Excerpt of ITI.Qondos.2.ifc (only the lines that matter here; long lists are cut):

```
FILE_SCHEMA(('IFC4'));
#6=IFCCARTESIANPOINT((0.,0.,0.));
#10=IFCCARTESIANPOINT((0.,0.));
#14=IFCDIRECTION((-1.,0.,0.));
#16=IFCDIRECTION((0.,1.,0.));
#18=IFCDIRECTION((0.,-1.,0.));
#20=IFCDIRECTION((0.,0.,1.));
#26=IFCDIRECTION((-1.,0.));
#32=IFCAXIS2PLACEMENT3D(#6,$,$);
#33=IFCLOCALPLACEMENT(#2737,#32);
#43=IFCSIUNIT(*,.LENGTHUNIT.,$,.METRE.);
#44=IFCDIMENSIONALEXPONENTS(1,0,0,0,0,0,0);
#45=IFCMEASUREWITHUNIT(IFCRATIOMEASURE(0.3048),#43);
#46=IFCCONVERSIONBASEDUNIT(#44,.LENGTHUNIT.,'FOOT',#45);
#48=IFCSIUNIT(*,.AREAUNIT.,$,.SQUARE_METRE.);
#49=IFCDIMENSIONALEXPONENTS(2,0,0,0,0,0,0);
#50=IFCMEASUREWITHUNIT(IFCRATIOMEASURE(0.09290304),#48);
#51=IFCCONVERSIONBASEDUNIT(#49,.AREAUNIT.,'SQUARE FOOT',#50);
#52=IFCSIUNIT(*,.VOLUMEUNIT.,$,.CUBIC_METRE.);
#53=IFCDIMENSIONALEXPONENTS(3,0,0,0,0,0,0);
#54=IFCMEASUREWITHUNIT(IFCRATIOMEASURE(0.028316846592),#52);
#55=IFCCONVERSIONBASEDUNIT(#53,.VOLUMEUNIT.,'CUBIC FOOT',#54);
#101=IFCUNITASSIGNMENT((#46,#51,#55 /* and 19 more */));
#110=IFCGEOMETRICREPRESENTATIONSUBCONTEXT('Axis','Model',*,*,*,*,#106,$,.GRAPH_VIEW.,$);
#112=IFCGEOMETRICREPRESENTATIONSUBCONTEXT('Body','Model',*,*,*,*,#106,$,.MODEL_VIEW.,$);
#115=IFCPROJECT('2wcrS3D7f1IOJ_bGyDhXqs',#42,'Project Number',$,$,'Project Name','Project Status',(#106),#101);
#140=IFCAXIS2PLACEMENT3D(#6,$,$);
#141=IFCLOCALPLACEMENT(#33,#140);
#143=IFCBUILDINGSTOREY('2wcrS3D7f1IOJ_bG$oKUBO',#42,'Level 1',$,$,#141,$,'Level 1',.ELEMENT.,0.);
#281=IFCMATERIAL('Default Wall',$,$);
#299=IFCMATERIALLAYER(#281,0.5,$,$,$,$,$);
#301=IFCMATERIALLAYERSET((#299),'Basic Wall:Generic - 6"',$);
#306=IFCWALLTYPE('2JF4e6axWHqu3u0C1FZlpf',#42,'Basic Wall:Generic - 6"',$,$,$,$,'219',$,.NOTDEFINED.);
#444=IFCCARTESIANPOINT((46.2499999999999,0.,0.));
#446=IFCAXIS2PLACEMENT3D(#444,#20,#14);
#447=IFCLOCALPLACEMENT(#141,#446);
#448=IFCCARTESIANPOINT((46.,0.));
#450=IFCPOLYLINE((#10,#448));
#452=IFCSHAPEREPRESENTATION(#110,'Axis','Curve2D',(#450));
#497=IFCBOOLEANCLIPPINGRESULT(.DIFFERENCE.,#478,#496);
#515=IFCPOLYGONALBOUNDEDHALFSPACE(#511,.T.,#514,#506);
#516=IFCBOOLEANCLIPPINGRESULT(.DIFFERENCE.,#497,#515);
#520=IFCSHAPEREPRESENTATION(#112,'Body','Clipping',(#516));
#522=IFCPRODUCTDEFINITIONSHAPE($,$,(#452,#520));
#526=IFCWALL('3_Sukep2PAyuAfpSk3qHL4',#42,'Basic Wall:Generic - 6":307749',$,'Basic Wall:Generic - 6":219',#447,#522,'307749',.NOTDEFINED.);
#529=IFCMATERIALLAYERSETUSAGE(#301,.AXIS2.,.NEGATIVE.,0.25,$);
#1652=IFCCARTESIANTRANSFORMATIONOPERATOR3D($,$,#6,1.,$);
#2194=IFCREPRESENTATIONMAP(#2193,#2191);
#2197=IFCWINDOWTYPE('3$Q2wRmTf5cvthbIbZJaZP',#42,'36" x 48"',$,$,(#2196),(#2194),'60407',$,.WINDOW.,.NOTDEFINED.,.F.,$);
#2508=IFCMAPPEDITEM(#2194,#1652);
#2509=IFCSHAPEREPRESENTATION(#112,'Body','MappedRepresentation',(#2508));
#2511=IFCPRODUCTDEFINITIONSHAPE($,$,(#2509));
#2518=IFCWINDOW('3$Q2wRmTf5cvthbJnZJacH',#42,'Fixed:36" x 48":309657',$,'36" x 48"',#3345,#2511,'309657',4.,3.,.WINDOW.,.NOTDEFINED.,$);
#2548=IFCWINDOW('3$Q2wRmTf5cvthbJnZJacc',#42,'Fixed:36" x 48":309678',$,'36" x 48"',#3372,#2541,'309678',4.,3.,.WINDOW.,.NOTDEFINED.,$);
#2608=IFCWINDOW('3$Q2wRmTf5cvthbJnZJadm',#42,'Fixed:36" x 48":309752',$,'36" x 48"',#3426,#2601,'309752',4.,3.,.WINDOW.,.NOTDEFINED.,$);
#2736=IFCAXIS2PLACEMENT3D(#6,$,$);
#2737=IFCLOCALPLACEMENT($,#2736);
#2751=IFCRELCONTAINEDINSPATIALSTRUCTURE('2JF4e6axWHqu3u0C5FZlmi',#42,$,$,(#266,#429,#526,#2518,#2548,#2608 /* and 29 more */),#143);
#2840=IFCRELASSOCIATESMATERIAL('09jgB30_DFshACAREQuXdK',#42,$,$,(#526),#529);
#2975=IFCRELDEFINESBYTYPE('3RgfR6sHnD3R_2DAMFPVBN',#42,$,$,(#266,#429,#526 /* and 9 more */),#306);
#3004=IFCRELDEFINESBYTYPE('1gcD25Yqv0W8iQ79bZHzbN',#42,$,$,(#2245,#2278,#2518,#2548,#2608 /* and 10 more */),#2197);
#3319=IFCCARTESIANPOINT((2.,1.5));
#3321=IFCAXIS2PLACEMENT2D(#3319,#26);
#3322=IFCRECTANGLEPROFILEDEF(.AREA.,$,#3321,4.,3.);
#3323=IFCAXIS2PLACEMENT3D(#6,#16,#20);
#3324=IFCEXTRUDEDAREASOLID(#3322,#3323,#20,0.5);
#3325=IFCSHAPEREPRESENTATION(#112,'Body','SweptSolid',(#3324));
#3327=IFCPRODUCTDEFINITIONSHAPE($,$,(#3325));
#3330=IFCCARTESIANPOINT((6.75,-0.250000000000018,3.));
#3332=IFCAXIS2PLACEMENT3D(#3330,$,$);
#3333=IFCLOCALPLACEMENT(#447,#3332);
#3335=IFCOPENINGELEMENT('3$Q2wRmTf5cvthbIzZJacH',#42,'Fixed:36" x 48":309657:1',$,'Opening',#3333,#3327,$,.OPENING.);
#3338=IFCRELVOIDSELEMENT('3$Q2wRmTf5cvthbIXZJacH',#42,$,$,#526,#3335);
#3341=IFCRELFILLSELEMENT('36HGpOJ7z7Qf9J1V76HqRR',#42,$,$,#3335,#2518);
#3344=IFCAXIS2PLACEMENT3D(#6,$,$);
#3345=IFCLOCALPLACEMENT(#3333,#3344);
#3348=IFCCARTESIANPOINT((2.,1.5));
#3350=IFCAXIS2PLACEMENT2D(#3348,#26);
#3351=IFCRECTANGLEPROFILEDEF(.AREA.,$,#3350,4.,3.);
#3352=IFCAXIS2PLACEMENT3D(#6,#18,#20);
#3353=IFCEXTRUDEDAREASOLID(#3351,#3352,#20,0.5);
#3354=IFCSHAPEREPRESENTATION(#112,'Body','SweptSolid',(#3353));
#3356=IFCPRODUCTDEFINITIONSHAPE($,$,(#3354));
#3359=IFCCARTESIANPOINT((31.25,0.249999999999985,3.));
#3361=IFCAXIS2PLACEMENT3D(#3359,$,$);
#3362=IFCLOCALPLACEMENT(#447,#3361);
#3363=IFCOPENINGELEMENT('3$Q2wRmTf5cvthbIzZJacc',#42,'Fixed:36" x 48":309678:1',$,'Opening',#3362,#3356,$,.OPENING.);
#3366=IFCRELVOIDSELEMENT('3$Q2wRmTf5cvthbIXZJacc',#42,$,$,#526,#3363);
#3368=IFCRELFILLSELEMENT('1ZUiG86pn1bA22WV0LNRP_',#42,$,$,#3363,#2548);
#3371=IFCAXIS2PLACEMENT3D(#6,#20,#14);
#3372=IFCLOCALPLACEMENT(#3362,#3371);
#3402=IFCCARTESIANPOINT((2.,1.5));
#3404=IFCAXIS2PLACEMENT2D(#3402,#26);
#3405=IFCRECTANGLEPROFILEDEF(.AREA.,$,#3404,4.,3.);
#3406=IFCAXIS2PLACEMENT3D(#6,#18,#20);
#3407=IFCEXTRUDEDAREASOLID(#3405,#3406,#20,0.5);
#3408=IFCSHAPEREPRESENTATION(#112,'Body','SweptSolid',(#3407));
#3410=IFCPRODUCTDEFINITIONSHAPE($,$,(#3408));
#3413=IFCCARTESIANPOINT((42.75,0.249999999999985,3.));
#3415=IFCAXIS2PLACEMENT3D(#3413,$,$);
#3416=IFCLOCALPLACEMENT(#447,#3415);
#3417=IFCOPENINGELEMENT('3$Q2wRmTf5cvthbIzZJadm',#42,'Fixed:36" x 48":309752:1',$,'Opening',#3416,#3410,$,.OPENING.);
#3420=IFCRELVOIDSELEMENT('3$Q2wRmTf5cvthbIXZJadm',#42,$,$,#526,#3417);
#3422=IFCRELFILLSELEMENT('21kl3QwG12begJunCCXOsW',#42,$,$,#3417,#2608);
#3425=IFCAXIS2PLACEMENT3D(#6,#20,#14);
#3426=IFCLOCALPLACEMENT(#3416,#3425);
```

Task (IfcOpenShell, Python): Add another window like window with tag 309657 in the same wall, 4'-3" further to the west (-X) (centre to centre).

```python
import ifcopenshell
import ifcopenshell.api.feature
import ifcopenshell.api.geometry
import ifcopenshell.api.root
import ifcopenshell.geom
import ifcopenshell.util.element
import ifcopenshell.util.placement
import ifcopenshell.util.shape
import ifcopenshell.util.unit

model = ifcopenshell.open("ITI.Qondos.2.ifc")
unit_scale = ifcopenshell.util.unit.calculate_unit_scale(model)
settings = ifcopenshell.geom.settings()


def volume(element):
    """Net volume in cubic metres, openings subtracted."""
    shape = ifcopenshell.geom.create_shape(settings, element)
    return ifcopenshell.util.shape.get_volume(shape.geometry)


def reuse_history(source, copy):
    """copy_class also copies each property set's owner history, people and application; keep the originals."""
    for rel in copy.IsDefinedBy:
        if rel.is_a("IfcRelDefinesByProperties") and (history := rel.RelatingPropertyDefinition.OwnerHistory):
            rel.RelatingPropertyDefinition.OwnerHistory = source.OwnerHistory
            ifcopenshell.util.element.remove_deep2(model, history)


window = model.by_guid("3$Q2wRmTf5cvthbJnZJacH")
opening = window.FillsVoids[0].RelatingOpeningElement
wall = opening.VoidsElements[0].RelatingBuildingElement
before = volume(wall)
shift = ifcopenshell.util.placement.get_local_placement(wall.ObjectPlacement)[:3, 0] * 51 * 0.0254 / unit_scale

# copy_class copies the void relationship, type, container and properties, but no geometry.
new_opening = ifcopenshell.api.root.copy_class(model, product=opening)
new_opening.Representation = ifcopenshell.util.element.copy_deep(
    model, opening.Representation, exclude=["IfcGeometricRepresentationContext", "IfcRepresentationMap"]
)
new_opening.Name = 'Fixed:36" x 48"'
new_window = ifcopenshell.api.root.copy_class(model, product=window)
new_window.Representation = ifcopenshell.util.element.copy_deep(
    model, window.Representation, exclude=["IfcGeometricRepresentationContext", "IfcRepresentationMap"]
)
new_window.Name = 'Fixed:36" x 48"'
new_window.Tag = None
reuse_history(window, new_window)
ifcopenshell.api.feature.add_filling(model, opening=new_opening, element=new_window)

for old, new in ((opening, new_opening), (window, new_window)):
    matrix = ifcopenshell.util.placement.get_local_placement(old.ObjectPlacement)
    matrix[:3, 3] += shift
    ifcopenshell.api.geometry.edit_object_placement(model, product=new, matrix=matrix, is_si=False)

after = volume(wall)

print(f"wall volume {before:.3f} -> {after:.3f} m3")

model.write("ITI.Qondos.2_updated.ifc")
```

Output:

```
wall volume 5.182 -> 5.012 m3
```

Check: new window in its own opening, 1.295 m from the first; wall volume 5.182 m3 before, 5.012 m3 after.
